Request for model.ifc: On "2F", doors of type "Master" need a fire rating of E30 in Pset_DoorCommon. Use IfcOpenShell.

First a look at what the model holds.

```python
import ifcopenshell
import ifcopenshell.util.element

model = ifcopenshell.open("model.ifc")
print(model.schema)
storey = next(s for s in model.by_type("IfcBuildingStorey") if s.Name == "2F")
doors = [e for e in ifcopenshell.util.element.get_decomposition(storey) if e.is_a("IfcDoor")]
seen = {}
for e in doors:
    element_type = ifcopenshell.util.element.get_type(e)
    key = (element_type.Name if element_type != e and element_type else None, ifcopenshell.util.element.get_pset(e, "Pset_DoorCommon", "FireRating"))
    seen[key] = seen.get(key, 0) + 1
for (name, value), count in sorted(seen.items(), key=str):
    print(count, "x", name, "|", value)
```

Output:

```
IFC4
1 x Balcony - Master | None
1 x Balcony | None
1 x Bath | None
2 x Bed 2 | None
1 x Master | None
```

```python
import ifcopenshell
import ifcopenshell.api.pset
import ifcopenshell.util.element

model = ifcopenshell.open("model.ifc")

storey = next(s for s in model.by_type("IfcBuildingStorey") if s.Name == "2F")
doors = [e for e in ifcopenshell.util.element.get_decomposition(storey) if e.is_a("IfcDoor")]

count = 0
for e in doors:
    element_type = ifcopenshell.util.element.get_type(e)
    if element_type in (None, e) or element_type.Name != "Master":
        continue
    # add_pset returns the element's existing set when there is one.
    pset = ifcopenshell.api.pset.add_pset(model, product=e, name="Pset_DoorCommon")
    ifcopenshell.api.pset.edit_pset(model, pset=pset, properties={"FireRating": "E30"})
    count += 1

print(count, "doors updated")

model.write("model_edited.ifc")
```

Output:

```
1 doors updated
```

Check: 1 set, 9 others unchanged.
